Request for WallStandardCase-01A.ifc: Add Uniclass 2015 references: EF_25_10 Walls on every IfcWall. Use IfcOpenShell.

First a look at what the model holds.

```python
import ifcopenshell

model = ifcopenshell.open("WallStandardCase-01A.ifc")
print(model.schema)
print("classifications:", [c.Name for c in model.by_type("IfcClassification")])
for ifc_class in ("IfcDoor", "IfcRoof", "IfcStair", "IfcWall", "IfcWindow"):
    print(ifc_class, len(model.by_type(ifc_class)))
```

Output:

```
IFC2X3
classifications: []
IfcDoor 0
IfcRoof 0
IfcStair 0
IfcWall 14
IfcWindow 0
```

```python
import ifcopenshell
import ifcopenshell.api.classification

model = ifcopenshell.open("WallStandardCase-01A.ifc")

# IFC2X3 requires Source and Edition and has no link from the project to the system.
system = model.create_entity("IfcClassification", Source="NBS", Edition="2015", Name="Uniclass 2015")

codes = {
    "IfcWall": ("EF_25_10", "Walls"),
}
for ifc_class, (code, name) in codes.items():
    products = model.by_type(ifc_class)
    ifcopenshell.api.classification.add_reference(
        model, products=products, classification=system, identification=code, name=name
    )
    print(code, len(products))

model.write("WallStandardCase-01A_updated.ifc")
```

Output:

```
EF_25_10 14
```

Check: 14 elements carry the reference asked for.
